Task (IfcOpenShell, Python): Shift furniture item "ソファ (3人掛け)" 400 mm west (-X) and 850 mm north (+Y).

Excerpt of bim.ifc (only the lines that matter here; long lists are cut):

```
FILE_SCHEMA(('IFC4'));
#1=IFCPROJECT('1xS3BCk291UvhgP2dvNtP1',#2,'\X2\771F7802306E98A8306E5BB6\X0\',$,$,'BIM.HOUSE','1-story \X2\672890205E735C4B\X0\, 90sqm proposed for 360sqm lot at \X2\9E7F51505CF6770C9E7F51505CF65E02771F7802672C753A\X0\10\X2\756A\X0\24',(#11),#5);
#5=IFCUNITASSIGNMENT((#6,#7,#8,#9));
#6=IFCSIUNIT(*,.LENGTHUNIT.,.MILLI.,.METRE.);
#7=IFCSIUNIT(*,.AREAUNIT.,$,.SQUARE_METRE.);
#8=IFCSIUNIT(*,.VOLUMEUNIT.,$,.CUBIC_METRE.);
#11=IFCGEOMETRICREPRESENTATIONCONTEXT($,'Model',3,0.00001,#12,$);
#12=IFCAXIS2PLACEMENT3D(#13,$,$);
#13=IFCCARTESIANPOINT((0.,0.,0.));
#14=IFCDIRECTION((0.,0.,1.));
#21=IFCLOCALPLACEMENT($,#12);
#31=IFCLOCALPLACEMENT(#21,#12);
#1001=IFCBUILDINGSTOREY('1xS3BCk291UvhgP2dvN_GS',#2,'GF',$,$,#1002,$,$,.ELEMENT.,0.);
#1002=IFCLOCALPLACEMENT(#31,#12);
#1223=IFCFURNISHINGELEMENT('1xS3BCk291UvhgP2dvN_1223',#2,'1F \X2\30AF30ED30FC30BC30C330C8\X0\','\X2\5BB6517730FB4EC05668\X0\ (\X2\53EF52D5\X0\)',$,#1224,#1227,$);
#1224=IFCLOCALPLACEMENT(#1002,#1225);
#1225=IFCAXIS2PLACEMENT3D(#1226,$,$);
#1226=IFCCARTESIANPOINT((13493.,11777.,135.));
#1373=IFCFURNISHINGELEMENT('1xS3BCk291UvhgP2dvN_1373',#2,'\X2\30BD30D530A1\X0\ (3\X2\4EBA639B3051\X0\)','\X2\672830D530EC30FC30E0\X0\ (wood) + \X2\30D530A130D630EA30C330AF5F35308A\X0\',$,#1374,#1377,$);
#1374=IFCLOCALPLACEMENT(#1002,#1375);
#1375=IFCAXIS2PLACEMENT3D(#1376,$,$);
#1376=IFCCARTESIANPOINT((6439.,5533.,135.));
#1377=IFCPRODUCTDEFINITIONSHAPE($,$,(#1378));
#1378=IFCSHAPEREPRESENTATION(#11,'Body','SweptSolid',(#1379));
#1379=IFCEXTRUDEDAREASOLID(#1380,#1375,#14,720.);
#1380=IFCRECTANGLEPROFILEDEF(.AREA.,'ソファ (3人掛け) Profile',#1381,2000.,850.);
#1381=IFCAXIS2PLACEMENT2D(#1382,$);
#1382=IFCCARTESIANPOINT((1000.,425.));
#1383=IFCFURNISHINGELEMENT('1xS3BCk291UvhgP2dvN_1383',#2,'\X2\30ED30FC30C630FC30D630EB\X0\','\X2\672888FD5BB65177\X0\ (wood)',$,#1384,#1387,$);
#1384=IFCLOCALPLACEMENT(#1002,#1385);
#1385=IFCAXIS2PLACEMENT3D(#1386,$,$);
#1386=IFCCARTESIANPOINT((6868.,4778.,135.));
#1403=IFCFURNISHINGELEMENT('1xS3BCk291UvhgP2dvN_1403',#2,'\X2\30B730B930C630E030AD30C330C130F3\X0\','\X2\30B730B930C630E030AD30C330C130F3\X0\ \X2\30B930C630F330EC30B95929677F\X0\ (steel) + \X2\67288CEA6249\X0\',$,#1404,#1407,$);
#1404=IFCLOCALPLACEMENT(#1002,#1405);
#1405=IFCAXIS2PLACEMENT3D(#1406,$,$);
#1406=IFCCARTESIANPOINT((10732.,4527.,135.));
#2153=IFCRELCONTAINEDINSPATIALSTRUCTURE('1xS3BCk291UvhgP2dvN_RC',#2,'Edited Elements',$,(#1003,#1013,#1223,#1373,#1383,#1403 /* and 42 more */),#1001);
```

```python
import ifcopenshell
import ifcopenshell.api.geometry
import ifcopenshell.util.placement
import ifcopenshell.util.unit

model = ifcopenshell.open("bim.ifc")
unit_scale = ifcopenshell.util.unit.calculate_unit_scale(model)

item = model.by_guid("1xS3BCk291UvhgP2dvN_1373")
matrix = ifcopenshell.util.placement.get_local_placement(item.ObjectPlacement)
matrix[0, 3] -= 0.4 / unit_scale
matrix[1, 3] += 0.85 / unit_scale
ifcopenshell.api.geometry.edit_object_placement(model, product=item, matrix=matrix, is_si=False)

print(ifcopenshell.util.placement.get_local_placement(item.ObjectPlacement).round(3) + 0.0)

model.write("bim_updated.ifc")
```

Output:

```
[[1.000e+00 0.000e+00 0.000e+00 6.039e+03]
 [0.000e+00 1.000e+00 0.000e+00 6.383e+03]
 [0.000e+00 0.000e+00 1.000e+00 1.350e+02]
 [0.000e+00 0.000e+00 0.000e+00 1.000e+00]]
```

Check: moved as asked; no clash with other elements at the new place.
